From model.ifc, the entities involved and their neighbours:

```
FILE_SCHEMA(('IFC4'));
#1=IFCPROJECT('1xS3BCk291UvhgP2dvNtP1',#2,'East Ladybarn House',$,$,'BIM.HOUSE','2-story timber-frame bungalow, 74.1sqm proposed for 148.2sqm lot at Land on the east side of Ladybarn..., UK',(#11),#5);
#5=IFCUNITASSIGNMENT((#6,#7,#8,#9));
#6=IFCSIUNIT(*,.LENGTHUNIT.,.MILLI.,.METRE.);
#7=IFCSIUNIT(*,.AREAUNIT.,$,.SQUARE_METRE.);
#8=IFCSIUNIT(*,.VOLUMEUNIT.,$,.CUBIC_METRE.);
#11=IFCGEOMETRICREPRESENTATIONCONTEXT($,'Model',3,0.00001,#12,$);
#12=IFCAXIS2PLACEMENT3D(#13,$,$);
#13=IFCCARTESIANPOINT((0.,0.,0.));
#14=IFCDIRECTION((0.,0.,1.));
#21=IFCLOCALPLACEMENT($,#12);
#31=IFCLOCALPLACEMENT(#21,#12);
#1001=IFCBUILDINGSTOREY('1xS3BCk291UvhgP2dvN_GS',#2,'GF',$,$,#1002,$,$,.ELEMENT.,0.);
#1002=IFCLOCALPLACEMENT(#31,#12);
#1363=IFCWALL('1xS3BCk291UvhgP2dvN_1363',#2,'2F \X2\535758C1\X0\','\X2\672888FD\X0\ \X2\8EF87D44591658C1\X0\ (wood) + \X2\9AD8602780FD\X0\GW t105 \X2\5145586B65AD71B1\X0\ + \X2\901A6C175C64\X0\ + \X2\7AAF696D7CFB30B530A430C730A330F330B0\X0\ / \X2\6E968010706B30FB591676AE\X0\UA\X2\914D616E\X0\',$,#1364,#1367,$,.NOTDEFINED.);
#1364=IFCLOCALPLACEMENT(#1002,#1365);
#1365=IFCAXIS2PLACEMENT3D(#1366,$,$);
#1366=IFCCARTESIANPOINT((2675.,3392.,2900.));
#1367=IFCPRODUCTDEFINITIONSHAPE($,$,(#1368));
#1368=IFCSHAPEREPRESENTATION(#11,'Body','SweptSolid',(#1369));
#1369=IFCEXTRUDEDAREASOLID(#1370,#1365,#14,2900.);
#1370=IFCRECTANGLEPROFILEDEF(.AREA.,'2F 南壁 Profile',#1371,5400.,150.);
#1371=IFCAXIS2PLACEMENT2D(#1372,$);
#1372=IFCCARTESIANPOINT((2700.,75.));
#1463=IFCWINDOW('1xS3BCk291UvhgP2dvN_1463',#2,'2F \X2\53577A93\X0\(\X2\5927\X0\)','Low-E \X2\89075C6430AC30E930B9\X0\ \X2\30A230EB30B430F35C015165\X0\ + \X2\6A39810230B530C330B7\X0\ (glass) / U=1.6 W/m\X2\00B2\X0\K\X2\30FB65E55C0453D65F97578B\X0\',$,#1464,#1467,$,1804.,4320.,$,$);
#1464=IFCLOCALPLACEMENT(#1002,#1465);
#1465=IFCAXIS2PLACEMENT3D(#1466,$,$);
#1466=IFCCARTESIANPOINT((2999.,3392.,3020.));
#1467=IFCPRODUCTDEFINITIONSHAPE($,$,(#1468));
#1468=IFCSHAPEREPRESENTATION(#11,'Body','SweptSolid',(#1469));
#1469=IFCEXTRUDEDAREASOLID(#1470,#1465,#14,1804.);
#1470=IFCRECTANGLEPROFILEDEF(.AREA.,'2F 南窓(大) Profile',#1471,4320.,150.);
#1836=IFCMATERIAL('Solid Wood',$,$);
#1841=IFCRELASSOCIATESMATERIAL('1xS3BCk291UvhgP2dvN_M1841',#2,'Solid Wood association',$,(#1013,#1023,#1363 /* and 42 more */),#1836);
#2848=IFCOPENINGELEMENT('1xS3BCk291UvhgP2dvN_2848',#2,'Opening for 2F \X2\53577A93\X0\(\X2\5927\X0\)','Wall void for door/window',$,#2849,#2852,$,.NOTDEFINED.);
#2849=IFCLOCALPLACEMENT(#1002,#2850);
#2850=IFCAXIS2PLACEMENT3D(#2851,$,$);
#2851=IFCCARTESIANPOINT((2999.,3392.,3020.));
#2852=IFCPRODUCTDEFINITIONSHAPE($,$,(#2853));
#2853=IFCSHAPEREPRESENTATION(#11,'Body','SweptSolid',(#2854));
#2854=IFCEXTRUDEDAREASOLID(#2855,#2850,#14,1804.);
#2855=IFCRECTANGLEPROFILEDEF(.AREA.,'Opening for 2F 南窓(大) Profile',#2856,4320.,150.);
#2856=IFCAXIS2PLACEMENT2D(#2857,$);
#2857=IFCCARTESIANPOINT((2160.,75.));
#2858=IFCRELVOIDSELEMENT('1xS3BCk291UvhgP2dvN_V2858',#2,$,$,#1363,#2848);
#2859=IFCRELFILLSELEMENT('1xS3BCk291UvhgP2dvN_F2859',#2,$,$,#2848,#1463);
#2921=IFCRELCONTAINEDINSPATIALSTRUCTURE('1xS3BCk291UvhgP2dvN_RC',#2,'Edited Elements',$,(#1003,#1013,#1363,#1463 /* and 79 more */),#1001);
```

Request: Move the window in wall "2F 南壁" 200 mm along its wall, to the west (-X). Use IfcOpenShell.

```python
import ifcopenshell
import ifcopenshell.api.geometry
import ifcopenshell.util.placement
import ifcopenshell.util.unit

model = ifcopenshell.open("model.ifc")
unit_scale = ifcopenshell.util.unit.calculate_unit_scale(model)

window = model.by_id(1463)
opening = window.FillsVoids[0].RelatingOpeningElement
wall = opening.VoidsElements[0].RelatingBuildingElement

wall_matrix = ifcopenshell.util.placement.get_local_placement(wall.ObjectPlacement)
shift = wall_matrix[:3, 0] * -0.2 / unit_scale
before = ifcopenshell.util.placement.get_local_placement(window.ObjectPlacement)[:3, 3].copy()

# The window is not placed relative to its opening, so move both.
for product in (opening, window):
    matrix = ifcopenshell.util.placement.get_local_placement(product.ObjectPlacement)
    matrix[:3, 3] += shift
    ifcopenshell.api.geometry.edit_object_placement(model, product=product, matrix=matrix, is_si=False)

after = ifcopenshell.util.placement.get_local_placement(window.ObjectPlacement)[:3, 3]
print("window moved by", (after - before).round(3) + 0.0)

model.write("model_updated.ifc")
```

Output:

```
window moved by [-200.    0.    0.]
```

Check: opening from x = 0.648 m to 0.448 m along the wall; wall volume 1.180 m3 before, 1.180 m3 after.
